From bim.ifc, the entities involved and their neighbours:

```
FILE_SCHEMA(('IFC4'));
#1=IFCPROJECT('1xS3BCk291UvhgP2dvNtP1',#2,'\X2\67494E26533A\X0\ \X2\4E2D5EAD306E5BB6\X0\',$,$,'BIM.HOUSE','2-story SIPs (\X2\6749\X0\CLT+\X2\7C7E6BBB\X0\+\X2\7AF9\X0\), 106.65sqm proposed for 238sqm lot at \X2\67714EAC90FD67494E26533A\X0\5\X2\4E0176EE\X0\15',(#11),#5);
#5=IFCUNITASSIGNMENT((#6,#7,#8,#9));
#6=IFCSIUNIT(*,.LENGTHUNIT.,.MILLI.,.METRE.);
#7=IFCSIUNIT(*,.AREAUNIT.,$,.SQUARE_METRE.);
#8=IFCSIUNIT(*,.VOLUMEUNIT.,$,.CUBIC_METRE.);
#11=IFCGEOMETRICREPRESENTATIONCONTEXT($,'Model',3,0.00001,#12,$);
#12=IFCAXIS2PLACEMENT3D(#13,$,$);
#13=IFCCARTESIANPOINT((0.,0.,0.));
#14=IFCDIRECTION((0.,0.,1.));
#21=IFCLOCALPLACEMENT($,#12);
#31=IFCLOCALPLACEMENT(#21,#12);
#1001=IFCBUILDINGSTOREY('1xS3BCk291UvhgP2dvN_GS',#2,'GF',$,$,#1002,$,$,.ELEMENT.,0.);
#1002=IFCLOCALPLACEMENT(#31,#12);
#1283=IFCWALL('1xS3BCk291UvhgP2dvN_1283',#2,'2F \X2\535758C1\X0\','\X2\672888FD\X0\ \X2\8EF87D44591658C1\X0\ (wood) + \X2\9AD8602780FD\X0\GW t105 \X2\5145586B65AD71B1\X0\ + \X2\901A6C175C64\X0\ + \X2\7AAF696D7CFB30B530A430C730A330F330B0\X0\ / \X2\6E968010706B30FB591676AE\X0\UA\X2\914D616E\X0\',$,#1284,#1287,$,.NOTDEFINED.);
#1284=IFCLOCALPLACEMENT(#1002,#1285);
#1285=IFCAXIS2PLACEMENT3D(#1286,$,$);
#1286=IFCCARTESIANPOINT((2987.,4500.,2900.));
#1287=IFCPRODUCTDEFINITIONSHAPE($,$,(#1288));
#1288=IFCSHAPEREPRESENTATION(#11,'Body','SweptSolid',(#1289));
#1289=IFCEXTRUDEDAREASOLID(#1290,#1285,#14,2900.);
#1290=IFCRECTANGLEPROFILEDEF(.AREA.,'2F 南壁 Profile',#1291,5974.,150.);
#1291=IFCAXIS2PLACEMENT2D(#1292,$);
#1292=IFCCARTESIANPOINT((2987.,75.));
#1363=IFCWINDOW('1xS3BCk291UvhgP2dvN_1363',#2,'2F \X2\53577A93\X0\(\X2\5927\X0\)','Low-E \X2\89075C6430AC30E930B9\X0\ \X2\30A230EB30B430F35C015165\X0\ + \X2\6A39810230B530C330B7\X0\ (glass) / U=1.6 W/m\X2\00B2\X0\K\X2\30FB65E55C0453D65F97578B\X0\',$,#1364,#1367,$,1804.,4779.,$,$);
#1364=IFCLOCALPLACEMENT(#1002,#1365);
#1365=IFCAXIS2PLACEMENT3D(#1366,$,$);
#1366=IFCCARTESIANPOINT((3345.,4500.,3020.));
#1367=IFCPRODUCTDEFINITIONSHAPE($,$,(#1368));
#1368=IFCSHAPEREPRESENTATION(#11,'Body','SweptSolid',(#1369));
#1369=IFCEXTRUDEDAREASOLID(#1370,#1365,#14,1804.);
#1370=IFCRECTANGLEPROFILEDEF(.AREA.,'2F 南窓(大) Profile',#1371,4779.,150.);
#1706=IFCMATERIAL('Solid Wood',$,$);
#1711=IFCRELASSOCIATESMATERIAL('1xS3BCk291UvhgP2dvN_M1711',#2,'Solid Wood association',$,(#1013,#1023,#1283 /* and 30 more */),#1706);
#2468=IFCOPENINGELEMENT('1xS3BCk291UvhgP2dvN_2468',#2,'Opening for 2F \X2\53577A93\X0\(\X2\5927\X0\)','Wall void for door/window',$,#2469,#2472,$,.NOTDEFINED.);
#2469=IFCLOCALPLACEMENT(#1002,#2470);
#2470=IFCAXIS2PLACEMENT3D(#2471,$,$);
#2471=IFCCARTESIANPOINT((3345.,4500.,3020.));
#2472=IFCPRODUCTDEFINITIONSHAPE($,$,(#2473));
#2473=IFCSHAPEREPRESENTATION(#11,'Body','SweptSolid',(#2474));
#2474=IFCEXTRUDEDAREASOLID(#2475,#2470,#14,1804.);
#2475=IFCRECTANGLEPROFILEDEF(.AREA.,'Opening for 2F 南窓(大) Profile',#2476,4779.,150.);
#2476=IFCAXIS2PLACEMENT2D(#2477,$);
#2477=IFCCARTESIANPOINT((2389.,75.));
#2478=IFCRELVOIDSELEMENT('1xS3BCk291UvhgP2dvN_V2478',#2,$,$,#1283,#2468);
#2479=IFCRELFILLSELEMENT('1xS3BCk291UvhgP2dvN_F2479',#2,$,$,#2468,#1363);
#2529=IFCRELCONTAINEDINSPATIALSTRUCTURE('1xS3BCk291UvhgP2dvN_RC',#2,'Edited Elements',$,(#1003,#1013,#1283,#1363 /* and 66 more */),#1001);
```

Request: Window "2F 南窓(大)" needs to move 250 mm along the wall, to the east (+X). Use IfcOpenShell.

```python
import ifcopenshell
import ifcopenshell.api.geometry
import ifcopenshell.util.placement
import ifcopenshell.util.unit

model = ifcopenshell.open("bim.ifc")
unit_scale = ifcopenshell.util.unit.calculate_unit_scale(model)

window = model.by_id(1363)
opening = window.FillsVoids[0].RelatingOpeningElement
wall = opening.VoidsElements[0].RelatingBuildingElement

wall_matrix = ifcopenshell.util.placement.get_local_placement(wall.ObjectPlacement)
shift = wall_matrix[:3, 0] * 0.25 / unit_scale
before = ifcopenshell.util.placement.get_local_placement(window.ObjectPlacement)[:3, 3].copy()

# The window is not placed relative to its opening, so move both.
for product in (opening, window):
    matrix = ifcopenshell.util.placement.get_local_placement(product.ObjectPlacement)
    matrix[:3, 3] += shift
    ifcopenshell.api.geometry.edit_object_placement(model, product=product, matrix=matrix, is_si=False)

after = ifcopenshell.util.placement.get_local_placement(window.ObjectPlacement)[:3, 3]
print("window moved by", (after - before).round(3) + 0.0)

model.write("bim_updated.ifc")
```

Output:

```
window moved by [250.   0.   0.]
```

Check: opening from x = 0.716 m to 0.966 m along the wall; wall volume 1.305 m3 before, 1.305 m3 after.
